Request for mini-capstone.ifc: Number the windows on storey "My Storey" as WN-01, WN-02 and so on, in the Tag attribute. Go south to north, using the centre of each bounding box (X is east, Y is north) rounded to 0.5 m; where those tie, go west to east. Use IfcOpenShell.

First a look at what the model holds.

```python
import ifcopenshell
import ifcopenshell.util.element
import ifcopenshell.util.placement

model = ifcopenshell.open("mini-capstone.ifc")
print(model.schema)
storey = next(s for s in model.by_type("IfcBuildingStorey") if s.Name == "My Storey")
windows = [e for e in ifcopenshell.util.element.get_decomposition(storey) if e.is_a("IfcWindow")]
for e in sorted(windows, key=lambda e: e.id()):
    origin = ifcopenshell.util.placement.get_local_placement(e.ObjectPlacement)[:3, 3]
    print(e.id(), e.Tag, e.Name, origin.round(2) + 0.0, sep=" | ")
```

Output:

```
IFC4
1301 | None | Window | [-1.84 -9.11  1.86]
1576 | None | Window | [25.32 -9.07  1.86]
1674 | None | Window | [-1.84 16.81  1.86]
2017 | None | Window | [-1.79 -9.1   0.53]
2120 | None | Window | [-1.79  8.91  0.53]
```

```python
import ifcopenshell
import ifcopenshell.geom
import ifcopenshell.util.element
import ifcopenshell.util.shape

model = ifcopenshell.open("mini-capstone.ifc")
settings = ifcopenshell.geom.settings()
settings.set("use-world-coords", True)


def centre(element):
    shape = ifcopenshell.geom.create_shape(settings, element)
    return ifcopenshell.util.shape.get_bbox_centroid(shape.geometry)


storey = next(s for s in model.by_type("IfcBuildingStorey") if s.Name == "My Storey")
windows = [e for e in ifcopenshell.util.element.get_decomposition(storey) if e.is_a("IfcWindow")]

# Insertion points can sit at a corner or the storey origin, so sort by the geometry (in metres).
centres = {e: centre(e) for e in windows}
windows.sort(key=lambda e: (round(centres[e][1] / 0.5), centres[e][0]))

for i, e in enumerate(windows, start=1):
    number = f"WN-{i:02d}"
    e.Tag = number
    print(e.id(), number)

model.write("mini-capstone_updated.ifc")
```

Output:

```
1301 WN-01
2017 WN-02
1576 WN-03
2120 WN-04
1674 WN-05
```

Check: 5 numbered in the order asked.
